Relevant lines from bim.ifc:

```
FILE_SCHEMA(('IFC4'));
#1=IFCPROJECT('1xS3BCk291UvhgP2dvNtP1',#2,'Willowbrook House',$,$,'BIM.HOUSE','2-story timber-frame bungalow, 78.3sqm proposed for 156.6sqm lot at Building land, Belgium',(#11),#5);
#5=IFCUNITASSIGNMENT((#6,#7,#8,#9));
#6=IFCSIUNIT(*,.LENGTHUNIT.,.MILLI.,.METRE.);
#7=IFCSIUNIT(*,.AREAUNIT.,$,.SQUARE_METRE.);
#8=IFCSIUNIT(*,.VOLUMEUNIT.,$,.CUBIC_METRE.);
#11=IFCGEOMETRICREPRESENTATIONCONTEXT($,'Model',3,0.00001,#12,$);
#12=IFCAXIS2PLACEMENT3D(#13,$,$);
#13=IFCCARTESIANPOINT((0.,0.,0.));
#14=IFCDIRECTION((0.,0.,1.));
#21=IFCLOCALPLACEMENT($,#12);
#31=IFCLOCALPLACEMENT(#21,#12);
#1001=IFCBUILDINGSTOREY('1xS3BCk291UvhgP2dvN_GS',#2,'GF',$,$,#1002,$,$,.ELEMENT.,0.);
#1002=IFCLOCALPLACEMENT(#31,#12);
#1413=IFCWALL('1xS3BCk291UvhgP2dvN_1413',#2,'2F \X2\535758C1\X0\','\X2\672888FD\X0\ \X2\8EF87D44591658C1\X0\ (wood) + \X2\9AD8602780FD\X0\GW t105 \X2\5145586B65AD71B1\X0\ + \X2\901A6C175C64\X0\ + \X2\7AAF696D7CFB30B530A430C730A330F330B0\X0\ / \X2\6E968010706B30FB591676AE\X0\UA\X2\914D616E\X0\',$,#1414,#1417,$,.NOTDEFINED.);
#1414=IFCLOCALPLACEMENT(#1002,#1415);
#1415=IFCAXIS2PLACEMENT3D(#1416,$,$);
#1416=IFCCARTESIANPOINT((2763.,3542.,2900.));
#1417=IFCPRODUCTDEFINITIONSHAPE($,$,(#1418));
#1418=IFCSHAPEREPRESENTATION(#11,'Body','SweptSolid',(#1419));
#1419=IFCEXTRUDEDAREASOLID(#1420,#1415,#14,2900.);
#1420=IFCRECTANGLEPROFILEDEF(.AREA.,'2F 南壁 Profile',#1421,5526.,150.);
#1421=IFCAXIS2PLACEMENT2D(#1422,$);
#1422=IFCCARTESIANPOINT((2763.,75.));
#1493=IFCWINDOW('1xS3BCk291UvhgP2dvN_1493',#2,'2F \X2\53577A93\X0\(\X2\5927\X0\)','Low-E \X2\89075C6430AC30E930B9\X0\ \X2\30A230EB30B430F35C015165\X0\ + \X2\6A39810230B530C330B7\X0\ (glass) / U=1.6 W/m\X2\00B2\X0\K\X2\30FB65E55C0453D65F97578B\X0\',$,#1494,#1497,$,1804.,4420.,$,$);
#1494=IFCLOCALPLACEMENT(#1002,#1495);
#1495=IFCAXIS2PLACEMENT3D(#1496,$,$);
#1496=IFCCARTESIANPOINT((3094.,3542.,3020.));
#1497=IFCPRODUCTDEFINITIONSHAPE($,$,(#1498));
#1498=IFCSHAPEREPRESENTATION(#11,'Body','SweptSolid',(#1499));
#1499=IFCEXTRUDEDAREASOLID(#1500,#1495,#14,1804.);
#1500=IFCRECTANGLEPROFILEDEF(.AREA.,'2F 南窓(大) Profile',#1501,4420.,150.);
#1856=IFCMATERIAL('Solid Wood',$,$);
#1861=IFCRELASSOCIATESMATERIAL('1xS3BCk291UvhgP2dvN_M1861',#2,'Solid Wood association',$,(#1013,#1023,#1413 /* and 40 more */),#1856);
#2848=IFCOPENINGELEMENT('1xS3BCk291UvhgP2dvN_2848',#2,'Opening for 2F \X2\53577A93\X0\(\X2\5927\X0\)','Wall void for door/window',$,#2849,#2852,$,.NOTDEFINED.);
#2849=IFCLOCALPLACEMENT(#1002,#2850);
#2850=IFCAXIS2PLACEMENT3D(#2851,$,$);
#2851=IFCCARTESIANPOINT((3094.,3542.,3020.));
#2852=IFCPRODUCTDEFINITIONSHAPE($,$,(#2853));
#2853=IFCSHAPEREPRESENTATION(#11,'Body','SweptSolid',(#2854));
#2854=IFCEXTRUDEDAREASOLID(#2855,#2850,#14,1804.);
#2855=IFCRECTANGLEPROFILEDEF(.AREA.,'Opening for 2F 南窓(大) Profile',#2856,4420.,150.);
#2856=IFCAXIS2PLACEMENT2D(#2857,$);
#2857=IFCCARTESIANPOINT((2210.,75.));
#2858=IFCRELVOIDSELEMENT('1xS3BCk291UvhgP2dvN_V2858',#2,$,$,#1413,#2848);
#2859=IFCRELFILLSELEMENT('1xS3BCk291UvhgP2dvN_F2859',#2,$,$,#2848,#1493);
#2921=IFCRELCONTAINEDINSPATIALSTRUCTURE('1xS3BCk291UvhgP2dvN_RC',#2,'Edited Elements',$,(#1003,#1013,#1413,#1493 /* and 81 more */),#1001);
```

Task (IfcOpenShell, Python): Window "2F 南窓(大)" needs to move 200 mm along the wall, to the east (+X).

```python
import ifcopenshell
import ifcopenshell.api.geometry
import ifcopenshell.util.placement

model = ifcopenshell.open("bim.ifc")

window = model.by_id(1493)
opening = window.FillsVoids[0].RelatingOpeningElement
wall = opening.VoidsElements[0].RelatingBuildingElement

wall_matrix = ifcopenshell.util.placement.get_local_placement(wall.ObjectPlacement)
shift = wall_matrix[:3, 0] * 200.0
before = ifcopenshell.util.placement.get_local_placement(window.ObjectPlacement)[:3, 3].copy()

# The window is not placed relative to its opening, so move both.
for product in (opening, window):
    matrix = ifcopenshell.util.placement.get_local_placement(product.ObjectPlacement)
    matrix[:3, 3] += shift
    ifcopenshell.api.geometry.edit_object_placement(model, product=product, matrix=matrix, is_si=False)

after = ifcopenshell.util.placement.get_local_placement(window.ObjectPlacement)[:3, 3]
print("window moved by", (after - before).round(3) + 0.0)

model.write("bim_v2.ifc")
```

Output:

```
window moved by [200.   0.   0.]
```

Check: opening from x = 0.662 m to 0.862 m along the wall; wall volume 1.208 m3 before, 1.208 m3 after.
